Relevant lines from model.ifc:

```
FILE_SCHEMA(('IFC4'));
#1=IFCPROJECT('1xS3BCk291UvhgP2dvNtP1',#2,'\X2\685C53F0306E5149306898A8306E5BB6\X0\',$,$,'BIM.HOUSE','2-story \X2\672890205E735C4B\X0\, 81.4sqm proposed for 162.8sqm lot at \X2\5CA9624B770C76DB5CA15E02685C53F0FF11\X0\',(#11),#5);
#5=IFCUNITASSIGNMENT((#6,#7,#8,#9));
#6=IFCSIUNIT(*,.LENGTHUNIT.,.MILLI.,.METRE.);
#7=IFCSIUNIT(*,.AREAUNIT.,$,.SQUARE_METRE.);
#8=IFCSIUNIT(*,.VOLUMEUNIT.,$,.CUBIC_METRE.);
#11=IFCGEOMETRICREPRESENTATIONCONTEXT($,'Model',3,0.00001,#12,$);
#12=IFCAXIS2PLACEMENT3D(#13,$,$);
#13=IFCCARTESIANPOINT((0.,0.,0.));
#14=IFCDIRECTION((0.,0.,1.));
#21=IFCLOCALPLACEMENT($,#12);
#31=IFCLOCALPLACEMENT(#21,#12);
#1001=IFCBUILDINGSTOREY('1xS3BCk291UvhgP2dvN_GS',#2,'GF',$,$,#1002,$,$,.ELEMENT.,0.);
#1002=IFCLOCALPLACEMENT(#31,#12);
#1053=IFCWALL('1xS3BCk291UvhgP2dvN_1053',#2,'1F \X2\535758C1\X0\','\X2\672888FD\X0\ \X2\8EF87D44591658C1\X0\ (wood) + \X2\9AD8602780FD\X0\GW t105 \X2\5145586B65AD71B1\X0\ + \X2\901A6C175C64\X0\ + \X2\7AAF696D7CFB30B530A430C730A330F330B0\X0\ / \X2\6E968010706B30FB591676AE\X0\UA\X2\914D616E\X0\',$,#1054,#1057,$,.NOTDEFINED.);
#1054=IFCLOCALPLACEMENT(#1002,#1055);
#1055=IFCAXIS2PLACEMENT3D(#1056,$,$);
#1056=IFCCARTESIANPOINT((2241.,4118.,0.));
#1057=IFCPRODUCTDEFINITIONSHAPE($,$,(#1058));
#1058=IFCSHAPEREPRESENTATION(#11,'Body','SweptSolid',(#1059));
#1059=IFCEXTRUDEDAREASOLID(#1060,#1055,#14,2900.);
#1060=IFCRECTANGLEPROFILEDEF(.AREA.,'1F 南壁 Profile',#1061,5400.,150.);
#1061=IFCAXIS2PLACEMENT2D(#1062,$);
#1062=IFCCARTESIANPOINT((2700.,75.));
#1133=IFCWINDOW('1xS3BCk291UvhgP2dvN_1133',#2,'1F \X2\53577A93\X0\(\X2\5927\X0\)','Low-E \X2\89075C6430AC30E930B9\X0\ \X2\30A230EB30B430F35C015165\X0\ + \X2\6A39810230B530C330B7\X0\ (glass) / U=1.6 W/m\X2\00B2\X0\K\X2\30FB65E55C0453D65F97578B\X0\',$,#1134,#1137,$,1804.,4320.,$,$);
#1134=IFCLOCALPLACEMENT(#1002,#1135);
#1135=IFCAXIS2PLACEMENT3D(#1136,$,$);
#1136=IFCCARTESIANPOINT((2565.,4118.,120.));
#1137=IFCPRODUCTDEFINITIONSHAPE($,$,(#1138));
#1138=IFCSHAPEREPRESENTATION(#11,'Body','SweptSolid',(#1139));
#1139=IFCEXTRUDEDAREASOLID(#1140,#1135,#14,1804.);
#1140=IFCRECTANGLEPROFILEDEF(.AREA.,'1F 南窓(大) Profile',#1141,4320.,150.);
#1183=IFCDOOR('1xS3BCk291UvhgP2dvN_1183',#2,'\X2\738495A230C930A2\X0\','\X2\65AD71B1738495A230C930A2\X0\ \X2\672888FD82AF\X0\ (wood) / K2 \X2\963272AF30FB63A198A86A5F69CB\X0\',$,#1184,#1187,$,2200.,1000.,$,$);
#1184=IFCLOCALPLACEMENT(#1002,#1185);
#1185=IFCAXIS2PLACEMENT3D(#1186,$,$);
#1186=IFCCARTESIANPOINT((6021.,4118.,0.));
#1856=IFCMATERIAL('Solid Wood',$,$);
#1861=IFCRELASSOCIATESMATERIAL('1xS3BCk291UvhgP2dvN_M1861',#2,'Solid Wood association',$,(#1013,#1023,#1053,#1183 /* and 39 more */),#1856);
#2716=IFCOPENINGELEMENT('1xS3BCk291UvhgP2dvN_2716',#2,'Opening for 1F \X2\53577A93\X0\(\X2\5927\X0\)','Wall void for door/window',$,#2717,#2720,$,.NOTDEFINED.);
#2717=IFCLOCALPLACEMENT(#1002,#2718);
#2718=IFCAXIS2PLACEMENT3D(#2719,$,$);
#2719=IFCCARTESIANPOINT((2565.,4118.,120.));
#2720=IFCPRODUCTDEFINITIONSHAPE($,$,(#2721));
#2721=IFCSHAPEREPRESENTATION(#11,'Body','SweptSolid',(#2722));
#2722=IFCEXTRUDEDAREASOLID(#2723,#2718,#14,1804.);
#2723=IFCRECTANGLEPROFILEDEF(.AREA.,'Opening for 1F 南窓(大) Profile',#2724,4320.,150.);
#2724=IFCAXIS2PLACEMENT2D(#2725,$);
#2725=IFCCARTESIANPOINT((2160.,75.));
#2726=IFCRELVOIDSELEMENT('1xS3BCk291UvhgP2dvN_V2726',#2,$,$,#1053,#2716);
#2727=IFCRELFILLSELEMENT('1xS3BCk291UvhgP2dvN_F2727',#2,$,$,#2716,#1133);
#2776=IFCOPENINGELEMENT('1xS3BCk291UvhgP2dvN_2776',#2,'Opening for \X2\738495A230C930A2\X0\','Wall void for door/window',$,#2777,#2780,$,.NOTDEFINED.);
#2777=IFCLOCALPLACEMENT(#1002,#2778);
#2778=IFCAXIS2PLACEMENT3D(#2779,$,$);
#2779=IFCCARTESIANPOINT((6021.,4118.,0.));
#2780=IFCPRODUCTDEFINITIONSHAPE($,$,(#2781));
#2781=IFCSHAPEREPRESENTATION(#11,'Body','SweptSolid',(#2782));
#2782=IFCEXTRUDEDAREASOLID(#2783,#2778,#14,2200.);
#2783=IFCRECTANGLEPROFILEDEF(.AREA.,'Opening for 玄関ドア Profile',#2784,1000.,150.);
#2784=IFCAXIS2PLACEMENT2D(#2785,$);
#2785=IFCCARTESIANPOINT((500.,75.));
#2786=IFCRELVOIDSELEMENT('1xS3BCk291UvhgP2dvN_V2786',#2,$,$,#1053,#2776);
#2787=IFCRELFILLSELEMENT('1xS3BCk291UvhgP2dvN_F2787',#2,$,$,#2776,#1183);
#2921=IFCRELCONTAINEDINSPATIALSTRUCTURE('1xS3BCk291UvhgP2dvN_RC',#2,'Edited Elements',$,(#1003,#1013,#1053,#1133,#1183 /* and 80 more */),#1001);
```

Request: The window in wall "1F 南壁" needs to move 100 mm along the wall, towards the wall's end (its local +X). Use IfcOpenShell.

```python
import ifcopenshell
import ifcopenshell.api.geometry
import ifcopenshell.util.placement
import ifcopenshell.util.unit

model = ifcopenshell.open("model.ifc")
unit_scale = ifcopenshell.util.unit.calculate_unit_scale(model)

window = model.by_guid("1xS3BCk291UvhgP2dvN_1133")
opening = window.FillsVoids[0].RelatingOpeningElement
wall = opening.VoidsElements[0].RelatingBuildingElement

wall_matrix = ifcopenshell.util.placement.get_local_placement(wall.ObjectPlacement)
shift = wall_matrix[:3, 0] * 0.1 / unit_scale
before = ifcopenshell.util.placement.get_local_placement(window.ObjectPlacement)[:3, 3].copy()

# The window is not placed relative to its opening, so move both.
for product in (opening, window):
    matrix = ifcopenshell.util.placement.get_local_placement(product.ObjectPlacement)
    matrix[:3, 3] += shift
    ifcopenshell.api.geometry.edit_object_placement(model, product=product, matrix=matrix, is_si=False)

after = ifcopenshell.util.placement.get_local_placement(window.ObjectPlacement)[:3, 3]
print("window moved by", (after - before).round(3) + 0.0)

model.write("model_edited.ifc")
```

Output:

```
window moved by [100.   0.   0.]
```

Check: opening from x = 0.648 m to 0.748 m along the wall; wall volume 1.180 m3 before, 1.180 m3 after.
